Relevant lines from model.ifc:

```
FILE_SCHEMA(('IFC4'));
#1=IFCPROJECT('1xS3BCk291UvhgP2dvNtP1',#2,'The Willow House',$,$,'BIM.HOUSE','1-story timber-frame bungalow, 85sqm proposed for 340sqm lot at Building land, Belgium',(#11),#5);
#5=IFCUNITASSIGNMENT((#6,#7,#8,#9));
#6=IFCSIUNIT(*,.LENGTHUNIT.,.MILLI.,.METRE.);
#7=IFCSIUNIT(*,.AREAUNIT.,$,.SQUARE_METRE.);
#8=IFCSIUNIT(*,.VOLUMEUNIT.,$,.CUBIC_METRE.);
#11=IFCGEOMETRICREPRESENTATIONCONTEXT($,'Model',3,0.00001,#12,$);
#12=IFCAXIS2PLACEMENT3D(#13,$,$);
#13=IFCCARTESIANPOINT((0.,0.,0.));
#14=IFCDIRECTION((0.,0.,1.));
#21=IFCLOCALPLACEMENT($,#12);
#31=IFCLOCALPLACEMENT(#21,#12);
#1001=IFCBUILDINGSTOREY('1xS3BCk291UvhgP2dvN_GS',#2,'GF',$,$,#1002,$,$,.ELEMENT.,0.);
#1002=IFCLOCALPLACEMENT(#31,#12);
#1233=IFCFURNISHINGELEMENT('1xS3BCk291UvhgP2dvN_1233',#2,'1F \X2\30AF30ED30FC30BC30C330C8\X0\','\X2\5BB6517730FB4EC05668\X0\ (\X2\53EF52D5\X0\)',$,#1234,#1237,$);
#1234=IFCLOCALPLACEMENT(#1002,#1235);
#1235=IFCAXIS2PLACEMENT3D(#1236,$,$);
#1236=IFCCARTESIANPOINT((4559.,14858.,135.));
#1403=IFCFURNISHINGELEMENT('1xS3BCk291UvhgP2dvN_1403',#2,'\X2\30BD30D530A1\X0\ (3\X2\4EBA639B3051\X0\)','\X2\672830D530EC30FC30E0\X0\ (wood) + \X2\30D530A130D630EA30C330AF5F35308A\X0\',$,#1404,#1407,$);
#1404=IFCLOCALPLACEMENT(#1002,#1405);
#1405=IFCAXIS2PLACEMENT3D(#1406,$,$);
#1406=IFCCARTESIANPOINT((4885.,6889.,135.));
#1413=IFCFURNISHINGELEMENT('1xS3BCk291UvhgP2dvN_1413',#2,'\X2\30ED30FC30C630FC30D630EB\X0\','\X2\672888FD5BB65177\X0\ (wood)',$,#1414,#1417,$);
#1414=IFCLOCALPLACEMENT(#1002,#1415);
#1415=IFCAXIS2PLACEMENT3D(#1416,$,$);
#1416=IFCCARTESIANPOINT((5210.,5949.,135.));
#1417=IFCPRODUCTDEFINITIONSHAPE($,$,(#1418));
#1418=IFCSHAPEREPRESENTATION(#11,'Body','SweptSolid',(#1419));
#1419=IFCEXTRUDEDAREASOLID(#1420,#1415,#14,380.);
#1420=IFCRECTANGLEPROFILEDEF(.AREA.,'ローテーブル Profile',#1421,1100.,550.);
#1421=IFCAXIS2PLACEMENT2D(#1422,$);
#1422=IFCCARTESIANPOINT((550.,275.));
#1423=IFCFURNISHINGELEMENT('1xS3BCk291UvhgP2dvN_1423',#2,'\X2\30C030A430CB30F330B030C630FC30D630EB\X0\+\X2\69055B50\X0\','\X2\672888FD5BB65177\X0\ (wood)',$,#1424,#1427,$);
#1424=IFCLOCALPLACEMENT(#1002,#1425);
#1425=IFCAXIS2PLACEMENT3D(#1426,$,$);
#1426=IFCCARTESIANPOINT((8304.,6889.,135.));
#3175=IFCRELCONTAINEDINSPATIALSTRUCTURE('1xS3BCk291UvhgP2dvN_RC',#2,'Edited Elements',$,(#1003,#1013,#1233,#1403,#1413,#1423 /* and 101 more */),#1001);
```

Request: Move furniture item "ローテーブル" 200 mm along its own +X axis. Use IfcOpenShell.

```python
import ifcopenshell
import ifcopenshell.api.geometry
import ifcopenshell.util.placement
import ifcopenshell.util.unit

model = ifcopenshell.open("model.ifc")
unit_scale = ifcopenshell.util.unit.calculate_unit_scale(model)

item = model.by_guid("1xS3BCk291UvhgP2dvN_1413")
matrix = ifcopenshell.util.placement.get_local_placement(item.ObjectPlacement)
matrix[:3, 3] += matrix[:3, 0] * 0.2 / unit_scale
ifcopenshell.api.geometry.edit_object_placement(model, product=item, matrix=matrix, is_si=False)

print(ifcopenshell.util.placement.get_local_placement(item.ObjectPlacement).round(3) + 0.0)

model.write("model_updated.ifc")
```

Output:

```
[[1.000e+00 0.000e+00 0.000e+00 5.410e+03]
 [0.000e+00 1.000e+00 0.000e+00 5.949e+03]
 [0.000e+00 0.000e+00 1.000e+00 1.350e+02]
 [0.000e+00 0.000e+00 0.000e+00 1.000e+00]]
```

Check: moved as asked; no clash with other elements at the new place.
